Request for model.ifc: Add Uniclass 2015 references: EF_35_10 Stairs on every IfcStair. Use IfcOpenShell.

First a look at what the model holds.

```python
import ifcopenshell

model = ifcopenshell.open("model.ifc")
print(model.schema)
print("classifications:", [c.Name for c in model.by_type("IfcClassification")])
for ifc_class in ("IfcDoor", "IfcRoof", "IfcStair", "IfcWall", "IfcWindow"):
    print(ifc_class, len(model.by_type(ifc_class)))
```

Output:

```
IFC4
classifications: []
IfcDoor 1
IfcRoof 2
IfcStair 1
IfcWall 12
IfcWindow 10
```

```python
import ifcopenshell
import ifcopenshell.api.classification

model = ifcopenshell.open("model.ifc")

system = ifcopenshell.api.classification.add_classification(model, classification="Uniclass 2015")

codes = {
    "IfcStair": ("EF_35_10", "Stairs"),
}
for ifc_class, (code, name) in codes.items():
    products = model.by_type(ifc_class)
    ifcopenshell.api.classification.add_reference(
        model, products=products, classification=system, identification=code, name=name
    )
    print(code, len(products))

model.write("model_rev.ifc")
```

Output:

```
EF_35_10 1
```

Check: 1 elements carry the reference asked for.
